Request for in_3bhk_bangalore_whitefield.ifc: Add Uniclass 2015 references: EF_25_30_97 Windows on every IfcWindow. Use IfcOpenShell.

First a look at what the model holds.

```python
import ifcopenshell

model = ifcopenshell.open("in_3bhk_bangalore_whitefield.ifc")
print(model.schema)
print("classifications:", [c.Name for c in model.by_type("IfcClassification")])
for ifc_class in ("IfcDoor", "IfcRoof", "IfcStair", "IfcWall", "IfcWindow"):
    print(ifc_class, len(model.by_type(ifc_class)))
```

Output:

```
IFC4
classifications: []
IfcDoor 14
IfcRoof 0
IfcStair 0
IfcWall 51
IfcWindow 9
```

```python
import ifcopenshell
import ifcopenshell.api.classification

model = ifcopenshell.open("in_3bhk_bangalore_whitefield.ifc")

system = ifcopenshell.api.classification.add_classification(model, classification="Uniclass 2015")

codes = {
    "IfcWindow": ("EF_25_30_97", "Windows"),
}
for ifc_class, (code, name) in codes.items():
    products = model.by_type(ifc_class)
    ifcopenshell.api.classification.add_reference(
        model, products=products, classification=system, identification=code, name=name
    )
    print(code, len(products))

model.write("in_3bhk_bangalore_whitefield_edited.ifc")
```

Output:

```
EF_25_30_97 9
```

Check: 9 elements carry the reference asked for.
